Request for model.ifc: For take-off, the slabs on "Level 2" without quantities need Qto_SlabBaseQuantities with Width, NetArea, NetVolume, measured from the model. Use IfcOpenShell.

First a look at what the model holds.

```python
import ifcopenshell
import ifcopenshell.util.element
import ifcopenshell.util.unit

model = ifcopenshell.open("model.ifc")
print(model.schema)
for unit_type in ("LENGTHUNIT", "AREAUNIT", "VOLUMEUNIT"):
    print(unit_type, ifcopenshell.util.unit.calculate_unit_scale(model, unit_type))
storey = next(s for s in model.by_type("IfcBuildingStorey") if s.Name == "Level 2")
slabs = [e for e in ifcopenshell.util.element.get_decomposition(storey) if e.is_a("IfcSlab")]
for e in sorted(slabs, key=lambda e: e.id()):
    print(e.id(), e.is_a(), e.Name, list(ifcopenshell.util.element.get_psets(e, qtos_only=True)), sep=" | ")
```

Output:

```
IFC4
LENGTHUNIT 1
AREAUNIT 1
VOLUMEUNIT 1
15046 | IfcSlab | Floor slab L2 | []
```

```python
import ifcopenshell
import ifcopenshell.api.pset
import ifcopenshell.geom
import ifcopenshell.util.element
import ifcopenshell.util.shape
import ifcopenshell.util.unit

model = ifcopenshell.open("model.ifc")
unit_scale = ifcopenshell.util.unit.calculate_unit_scale(model)
area_scale = ifcopenshell.util.unit.calculate_unit_scale(model, "AREAUNIT")
volume_scale = ifcopenshell.util.unit.calculate_unit_scale(model, "VOLUMEUNIT")
settings = ifcopenshell.geom.settings()

storey = next(s for s in model.by_type("IfcBuildingStorey") if s.Name == "Level 2")
slabs = [e for e in ifcopenshell.util.element.get_decomposition(storey) if e.is_a("IfcSlab")]

for e in sorted(slabs, key=lambda e: e.id()):
    if ifcopenshell.util.element.get_psets(e, qtos_only=True, should_inherit=False):
        continue
    # Geometry comes back in metres, in the element's own axes.
    shape = ifcopenshell.geom.create_shape(settings, e)
    values = {
        "Width": ifcopenshell.util.shape.get_z(shape.geometry) / unit_scale,
        "NetArea": ifcopenshell.util.shape.get_footprint_area(shape.geometry) / area_scale,
        "NetVolume": ifcopenshell.util.shape.get_volume(shape.geometry) / volume_scale,
    }
    qto = ifcopenshell.api.pset.add_qto(model, product=e, name="Qto_SlabBaseQuantities")
    ifcopenshell.api.pset.edit_qto(model, qto=qto, properties=values)
    print(e.id(), {k: round(v, 3) for k, v in values.items()})

model.write("model_rev.ifc")
```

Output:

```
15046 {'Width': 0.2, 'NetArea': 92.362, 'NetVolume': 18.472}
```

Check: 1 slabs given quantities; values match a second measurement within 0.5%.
